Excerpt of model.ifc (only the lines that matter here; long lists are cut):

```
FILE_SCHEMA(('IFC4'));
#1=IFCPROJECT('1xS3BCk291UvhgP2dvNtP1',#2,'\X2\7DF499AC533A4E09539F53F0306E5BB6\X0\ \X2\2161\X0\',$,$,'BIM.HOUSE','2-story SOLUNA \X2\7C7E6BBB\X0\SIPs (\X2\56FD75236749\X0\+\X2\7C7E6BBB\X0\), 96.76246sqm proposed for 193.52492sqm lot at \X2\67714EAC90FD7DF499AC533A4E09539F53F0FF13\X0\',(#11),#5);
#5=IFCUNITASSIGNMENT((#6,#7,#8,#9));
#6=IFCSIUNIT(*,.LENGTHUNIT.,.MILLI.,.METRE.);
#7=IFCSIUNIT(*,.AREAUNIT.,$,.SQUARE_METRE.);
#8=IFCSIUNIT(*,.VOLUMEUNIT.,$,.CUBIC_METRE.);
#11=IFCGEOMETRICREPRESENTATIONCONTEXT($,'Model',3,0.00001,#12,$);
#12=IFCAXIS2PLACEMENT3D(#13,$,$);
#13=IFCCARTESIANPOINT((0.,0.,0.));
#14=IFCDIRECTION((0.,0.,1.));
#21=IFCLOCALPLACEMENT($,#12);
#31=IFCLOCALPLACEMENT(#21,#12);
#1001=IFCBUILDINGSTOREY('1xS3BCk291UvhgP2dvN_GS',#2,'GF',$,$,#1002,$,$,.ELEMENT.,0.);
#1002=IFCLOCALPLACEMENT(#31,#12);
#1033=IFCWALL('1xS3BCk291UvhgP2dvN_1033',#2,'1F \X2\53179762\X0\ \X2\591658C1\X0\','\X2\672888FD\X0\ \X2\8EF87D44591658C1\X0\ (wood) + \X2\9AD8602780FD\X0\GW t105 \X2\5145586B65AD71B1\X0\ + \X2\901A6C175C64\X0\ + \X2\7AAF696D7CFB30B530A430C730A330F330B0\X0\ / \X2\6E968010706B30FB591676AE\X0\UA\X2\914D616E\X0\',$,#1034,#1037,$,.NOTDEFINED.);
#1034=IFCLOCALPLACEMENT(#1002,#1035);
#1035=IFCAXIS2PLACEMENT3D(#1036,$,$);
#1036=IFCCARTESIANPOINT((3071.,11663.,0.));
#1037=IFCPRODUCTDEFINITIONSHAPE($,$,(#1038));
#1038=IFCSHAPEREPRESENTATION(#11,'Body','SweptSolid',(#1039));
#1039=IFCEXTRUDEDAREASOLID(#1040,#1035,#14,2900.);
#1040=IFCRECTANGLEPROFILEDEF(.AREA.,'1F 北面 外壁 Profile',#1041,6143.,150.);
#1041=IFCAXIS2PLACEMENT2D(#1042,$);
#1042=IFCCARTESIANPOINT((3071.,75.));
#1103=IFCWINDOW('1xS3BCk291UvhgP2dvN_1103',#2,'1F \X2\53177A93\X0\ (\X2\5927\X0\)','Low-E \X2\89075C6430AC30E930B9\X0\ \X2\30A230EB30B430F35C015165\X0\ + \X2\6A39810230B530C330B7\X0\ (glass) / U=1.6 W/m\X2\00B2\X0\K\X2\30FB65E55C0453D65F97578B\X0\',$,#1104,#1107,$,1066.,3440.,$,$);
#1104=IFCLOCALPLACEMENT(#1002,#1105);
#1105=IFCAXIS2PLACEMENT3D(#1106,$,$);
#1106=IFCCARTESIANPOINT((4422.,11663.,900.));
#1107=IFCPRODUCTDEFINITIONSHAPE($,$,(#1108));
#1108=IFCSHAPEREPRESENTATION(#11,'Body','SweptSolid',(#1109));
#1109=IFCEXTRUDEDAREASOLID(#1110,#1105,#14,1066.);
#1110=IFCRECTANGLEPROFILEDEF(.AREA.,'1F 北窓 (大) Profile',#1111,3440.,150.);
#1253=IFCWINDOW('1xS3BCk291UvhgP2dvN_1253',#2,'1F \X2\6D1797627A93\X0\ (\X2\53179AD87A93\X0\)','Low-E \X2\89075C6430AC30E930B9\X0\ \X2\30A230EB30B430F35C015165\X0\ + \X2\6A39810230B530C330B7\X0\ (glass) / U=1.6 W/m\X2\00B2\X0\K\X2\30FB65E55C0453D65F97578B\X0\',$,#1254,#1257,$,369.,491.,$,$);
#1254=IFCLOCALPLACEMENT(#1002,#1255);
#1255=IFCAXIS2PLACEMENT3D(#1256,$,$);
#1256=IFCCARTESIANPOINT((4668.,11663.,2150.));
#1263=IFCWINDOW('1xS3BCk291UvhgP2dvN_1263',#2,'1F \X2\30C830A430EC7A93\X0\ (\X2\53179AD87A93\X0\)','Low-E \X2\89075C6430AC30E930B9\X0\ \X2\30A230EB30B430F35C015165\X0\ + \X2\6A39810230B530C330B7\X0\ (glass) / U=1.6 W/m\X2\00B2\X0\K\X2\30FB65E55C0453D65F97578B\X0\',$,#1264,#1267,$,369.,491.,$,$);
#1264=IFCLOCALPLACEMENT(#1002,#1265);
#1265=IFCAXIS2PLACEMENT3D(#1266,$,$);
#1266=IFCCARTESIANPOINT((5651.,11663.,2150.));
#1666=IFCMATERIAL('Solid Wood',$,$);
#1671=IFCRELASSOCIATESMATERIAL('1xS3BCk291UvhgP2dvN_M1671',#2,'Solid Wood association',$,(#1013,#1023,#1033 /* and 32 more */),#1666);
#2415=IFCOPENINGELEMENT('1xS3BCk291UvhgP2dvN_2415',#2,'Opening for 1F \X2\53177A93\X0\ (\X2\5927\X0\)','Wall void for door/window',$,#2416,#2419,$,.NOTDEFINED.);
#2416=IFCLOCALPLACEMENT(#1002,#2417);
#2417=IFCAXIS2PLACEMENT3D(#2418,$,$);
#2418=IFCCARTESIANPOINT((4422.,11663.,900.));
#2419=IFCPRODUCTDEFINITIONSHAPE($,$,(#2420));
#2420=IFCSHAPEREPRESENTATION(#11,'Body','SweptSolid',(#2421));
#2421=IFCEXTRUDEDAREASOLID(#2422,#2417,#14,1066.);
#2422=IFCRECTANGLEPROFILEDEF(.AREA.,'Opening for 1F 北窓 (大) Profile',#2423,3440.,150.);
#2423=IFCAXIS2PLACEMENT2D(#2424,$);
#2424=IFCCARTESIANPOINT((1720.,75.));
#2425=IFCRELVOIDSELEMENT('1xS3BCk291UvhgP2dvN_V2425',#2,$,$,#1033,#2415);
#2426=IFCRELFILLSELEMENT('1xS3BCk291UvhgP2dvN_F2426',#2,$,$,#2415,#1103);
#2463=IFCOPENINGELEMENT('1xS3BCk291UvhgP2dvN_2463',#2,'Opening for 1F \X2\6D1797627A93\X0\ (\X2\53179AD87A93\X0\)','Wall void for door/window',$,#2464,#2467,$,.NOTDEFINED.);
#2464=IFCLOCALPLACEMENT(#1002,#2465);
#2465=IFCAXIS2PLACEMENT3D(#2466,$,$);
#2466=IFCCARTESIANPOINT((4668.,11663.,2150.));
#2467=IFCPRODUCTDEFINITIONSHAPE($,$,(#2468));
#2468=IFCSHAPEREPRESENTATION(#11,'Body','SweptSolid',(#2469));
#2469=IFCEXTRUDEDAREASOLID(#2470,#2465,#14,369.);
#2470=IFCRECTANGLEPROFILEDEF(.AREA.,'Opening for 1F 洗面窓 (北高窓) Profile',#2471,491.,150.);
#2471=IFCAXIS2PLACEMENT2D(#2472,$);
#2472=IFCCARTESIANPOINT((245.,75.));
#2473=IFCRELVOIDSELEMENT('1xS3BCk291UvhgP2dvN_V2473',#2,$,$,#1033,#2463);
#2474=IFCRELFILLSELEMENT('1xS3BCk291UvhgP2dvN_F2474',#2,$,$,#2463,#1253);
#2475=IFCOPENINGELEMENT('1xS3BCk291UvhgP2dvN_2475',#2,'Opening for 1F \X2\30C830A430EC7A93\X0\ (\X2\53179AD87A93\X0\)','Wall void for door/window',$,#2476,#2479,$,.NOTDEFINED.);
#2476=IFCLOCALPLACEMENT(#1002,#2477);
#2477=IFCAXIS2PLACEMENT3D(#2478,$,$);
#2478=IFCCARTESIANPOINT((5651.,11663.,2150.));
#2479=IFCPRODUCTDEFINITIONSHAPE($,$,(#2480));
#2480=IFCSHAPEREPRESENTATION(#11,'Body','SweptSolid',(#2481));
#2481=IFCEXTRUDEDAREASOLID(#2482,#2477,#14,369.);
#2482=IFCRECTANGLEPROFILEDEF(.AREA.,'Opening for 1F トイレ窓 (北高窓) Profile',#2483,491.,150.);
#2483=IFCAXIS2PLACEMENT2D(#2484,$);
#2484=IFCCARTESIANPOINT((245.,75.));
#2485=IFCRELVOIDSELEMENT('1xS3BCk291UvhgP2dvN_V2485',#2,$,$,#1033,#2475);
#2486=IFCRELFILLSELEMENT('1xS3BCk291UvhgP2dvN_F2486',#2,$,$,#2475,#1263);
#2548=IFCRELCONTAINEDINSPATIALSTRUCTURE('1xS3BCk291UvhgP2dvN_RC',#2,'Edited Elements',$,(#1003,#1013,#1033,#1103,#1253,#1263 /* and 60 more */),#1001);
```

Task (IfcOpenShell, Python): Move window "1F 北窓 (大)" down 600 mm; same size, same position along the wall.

```python
import numpy as np
import ifcopenshell
import ifcopenshell.api.geometry
import ifcopenshell.util.placement
import ifcopenshell.util.unit

model = ifcopenshell.open("model.ifc")
unit_scale = ifcopenshell.util.unit.calculate_unit_scale(model)

window = model.by_guid("1xS3BCk291UvhgP2dvN_1103")
opening = window.FillsVoids[0].RelatingOpeningElement
dz = -0.6 / unit_scale

shift = np.array([0.0, 0.0, dz])
# The window is not placed relative to its opening, so move both.
for product in (opening, window):
    matrix = ifcopenshell.util.placement.get_local_placement(product.ObjectPlacement)
    matrix[:3, 3] += shift
    ifcopenshell.api.geometry.edit_object_placement(model, product=product, matrix=matrix, is_si=False)

print(f"moved by {dz * unit_scale:+.3f} m")

model.write("model_rev.ifc")
```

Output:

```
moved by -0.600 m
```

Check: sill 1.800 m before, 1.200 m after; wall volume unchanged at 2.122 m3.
